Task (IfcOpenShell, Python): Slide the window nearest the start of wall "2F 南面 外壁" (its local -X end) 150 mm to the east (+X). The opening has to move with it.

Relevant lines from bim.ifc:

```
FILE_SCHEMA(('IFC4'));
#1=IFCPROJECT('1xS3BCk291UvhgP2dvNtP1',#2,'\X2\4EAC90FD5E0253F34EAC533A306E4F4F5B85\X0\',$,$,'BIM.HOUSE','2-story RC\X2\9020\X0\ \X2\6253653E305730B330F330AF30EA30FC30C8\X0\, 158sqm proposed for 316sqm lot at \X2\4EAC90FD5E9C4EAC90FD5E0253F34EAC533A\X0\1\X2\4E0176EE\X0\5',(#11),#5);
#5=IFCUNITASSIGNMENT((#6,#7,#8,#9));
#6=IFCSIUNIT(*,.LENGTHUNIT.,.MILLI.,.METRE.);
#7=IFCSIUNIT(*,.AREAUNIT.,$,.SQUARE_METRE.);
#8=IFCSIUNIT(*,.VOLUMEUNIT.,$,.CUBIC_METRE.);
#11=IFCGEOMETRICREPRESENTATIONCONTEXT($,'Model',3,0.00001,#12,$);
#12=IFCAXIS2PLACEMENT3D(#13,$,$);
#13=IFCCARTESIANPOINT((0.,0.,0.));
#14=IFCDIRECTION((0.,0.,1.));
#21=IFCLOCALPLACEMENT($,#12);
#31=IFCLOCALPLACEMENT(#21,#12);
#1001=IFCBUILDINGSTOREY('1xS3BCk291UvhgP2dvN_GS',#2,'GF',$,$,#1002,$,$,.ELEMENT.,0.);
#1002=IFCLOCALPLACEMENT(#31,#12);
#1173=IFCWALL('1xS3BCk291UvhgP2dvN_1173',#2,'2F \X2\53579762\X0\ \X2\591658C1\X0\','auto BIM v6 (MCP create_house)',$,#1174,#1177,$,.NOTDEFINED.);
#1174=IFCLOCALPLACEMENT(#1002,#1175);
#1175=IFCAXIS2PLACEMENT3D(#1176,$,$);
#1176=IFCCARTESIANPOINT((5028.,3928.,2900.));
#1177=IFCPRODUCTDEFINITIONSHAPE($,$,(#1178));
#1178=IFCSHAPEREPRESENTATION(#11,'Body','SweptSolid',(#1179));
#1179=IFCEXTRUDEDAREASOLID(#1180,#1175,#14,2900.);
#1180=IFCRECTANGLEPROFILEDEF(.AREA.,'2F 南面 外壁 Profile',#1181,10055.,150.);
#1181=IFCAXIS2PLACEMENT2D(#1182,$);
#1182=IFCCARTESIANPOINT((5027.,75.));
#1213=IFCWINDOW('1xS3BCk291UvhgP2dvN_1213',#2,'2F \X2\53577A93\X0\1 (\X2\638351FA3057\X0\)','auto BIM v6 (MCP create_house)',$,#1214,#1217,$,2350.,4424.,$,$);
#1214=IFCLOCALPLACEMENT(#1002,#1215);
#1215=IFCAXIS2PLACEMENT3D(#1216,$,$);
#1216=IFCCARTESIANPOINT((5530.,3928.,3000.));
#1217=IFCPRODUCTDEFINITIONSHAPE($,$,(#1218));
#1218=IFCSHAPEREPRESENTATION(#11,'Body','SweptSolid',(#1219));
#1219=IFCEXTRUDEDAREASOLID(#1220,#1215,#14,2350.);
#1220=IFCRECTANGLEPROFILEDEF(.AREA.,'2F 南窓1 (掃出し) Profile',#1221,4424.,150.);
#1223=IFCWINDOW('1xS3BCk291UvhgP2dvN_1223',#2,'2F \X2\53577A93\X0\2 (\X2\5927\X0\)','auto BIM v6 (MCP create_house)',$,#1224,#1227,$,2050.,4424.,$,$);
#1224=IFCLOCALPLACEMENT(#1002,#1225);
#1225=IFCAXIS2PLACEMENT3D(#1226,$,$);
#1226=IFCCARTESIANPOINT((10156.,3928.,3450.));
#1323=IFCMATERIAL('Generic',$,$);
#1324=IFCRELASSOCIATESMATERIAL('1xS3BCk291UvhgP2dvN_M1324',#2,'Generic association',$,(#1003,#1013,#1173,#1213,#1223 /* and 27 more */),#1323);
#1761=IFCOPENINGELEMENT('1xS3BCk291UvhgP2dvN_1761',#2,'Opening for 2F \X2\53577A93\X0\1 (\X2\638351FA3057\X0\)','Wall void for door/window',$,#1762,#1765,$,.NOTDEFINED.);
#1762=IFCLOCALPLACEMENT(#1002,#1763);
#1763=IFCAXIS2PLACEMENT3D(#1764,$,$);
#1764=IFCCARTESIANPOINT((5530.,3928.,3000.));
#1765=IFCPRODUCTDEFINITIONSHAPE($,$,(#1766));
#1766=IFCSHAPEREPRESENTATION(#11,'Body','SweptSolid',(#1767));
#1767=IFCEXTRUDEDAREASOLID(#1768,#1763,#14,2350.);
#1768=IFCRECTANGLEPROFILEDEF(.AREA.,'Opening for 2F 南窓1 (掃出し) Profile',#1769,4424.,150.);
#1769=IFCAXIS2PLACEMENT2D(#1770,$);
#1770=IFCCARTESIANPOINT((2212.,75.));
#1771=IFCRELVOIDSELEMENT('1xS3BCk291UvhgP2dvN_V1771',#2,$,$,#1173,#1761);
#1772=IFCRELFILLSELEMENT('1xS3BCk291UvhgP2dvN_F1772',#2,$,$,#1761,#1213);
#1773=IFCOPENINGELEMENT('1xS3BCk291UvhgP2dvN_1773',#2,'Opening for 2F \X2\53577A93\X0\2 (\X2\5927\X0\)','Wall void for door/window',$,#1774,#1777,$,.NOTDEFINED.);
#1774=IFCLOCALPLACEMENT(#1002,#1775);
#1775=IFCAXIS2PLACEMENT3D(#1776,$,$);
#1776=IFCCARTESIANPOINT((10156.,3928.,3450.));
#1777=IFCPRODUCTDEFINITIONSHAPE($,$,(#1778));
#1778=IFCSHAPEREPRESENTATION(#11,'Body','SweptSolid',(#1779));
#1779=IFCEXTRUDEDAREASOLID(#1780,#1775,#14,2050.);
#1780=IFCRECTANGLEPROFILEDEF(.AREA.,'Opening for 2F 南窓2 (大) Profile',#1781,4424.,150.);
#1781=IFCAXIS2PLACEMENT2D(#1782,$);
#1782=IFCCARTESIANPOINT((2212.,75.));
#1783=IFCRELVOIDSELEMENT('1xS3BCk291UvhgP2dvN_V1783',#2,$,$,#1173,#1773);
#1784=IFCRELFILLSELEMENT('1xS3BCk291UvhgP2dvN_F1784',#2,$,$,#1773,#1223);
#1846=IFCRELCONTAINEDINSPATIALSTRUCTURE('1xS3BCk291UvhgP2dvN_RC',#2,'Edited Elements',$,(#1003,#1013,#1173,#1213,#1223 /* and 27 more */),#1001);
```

```python
import ifcopenshell
import ifcopenshell.api.geometry
import ifcopenshell.util.placement
import ifcopenshell.util.unit

model = ifcopenshell.open("bim.ifc")
unit_scale = ifcopenshell.util.unit.calculate_unit_scale(model)

window = model.by_guid("1xS3BCk291UvhgP2dvN_1213")
opening = window.FillsVoids[0].RelatingOpeningElement
wall = opening.VoidsElements[0].RelatingBuildingElement

wall_matrix = ifcopenshell.util.placement.get_local_placement(wall.ObjectPlacement)
shift = wall_matrix[:3, 0] * 0.15 / unit_scale
before = ifcopenshell.util.placement.get_local_placement(window.ObjectPlacement)[:3, 3].copy()

# The window is not placed relative to its opening, so move both.
for product in (opening, window):
    matrix = ifcopenshell.util.placement.get_local_placement(product.ObjectPlacement)
    matrix[:3, 3] += shift
    ifcopenshell.api.geometry.edit_object_placement(model, product=product, matrix=matrix, is_si=False)

after = ifcopenshell.util.placement.get_local_placement(window.ObjectPlacement)[:3, 3]
print("window moved by", (after - before).round(3) + 0.0)

model.write("bim-out.ifc")
```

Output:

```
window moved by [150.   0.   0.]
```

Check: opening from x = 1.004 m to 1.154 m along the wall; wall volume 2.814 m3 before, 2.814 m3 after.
